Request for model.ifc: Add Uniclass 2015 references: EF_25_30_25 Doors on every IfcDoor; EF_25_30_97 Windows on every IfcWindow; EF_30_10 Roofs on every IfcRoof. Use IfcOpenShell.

First a look at what the model holds.

```python
import ifcopenshell

model = ifcopenshell.open("model.ifc")
print(model.schema)
print("classifications:", [c.Name for c in model.by_type("IfcClassification")])
for ifc_class in ("IfcDoor", "IfcRoof", "IfcStair", "IfcWall", "IfcWindow"):
    print(ifc_class, len(model.by_type(ifc_class)))
```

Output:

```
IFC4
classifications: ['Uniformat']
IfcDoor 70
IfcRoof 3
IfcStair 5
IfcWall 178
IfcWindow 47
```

```python
import ifcopenshell
import ifcopenshell.api.classification

model = ifcopenshell.open("model.ifc")

system = ifcopenshell.api.classification.add_classification(model, classification="Uniclass 2015")

codes = {
    "IfcDoor": ("EF_25_30_25", "Doors"),
    "IfcWindow": ("EF_25_30_97", "Windows"),
    "IfcRoof": ("EF_30_10", "Roofs"),
}
for ifc_class, (code, name) in codes.items():
    products = model.by_type(ifc_class)
    ifcopenshell.api.classification.add_reference(
        model, products=products, classification=system, identification=code, name=name
    )
    print(code, len(products))

model.write("model_rev.ifc")
```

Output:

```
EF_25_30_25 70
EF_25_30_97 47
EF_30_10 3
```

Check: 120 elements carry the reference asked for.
